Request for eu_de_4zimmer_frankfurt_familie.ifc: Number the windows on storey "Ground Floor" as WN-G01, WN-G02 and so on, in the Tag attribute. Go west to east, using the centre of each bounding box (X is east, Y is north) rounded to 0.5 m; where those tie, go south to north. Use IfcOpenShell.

First a look at what the model holds.

```python
import ifcopenshell
import ifcopenshell.util.element
import ifcopenshell.util.placement

model = ifcopenshell.open("eu_de_4zimmer_frankfurt_familie.ifc")
print(model.schema)
storey = next(s for s in model.by_type("IfcBuildingStorey") if s.Name == "Ground Floor")
windows = [e for e in ifcopenshell.util.element.get_decomposition(storey) if e.is_a("IfcWindow")]
for e in sorted(windows, key=lambda e: e.id()):
    origin = ifcopenshell.util.placement.get_local_placement(e.ObjectPlacement)[:3, 3]
    print(e.id(), e.Tag, e.Name, origin.round(2) + 0.0, sep=" | ")
```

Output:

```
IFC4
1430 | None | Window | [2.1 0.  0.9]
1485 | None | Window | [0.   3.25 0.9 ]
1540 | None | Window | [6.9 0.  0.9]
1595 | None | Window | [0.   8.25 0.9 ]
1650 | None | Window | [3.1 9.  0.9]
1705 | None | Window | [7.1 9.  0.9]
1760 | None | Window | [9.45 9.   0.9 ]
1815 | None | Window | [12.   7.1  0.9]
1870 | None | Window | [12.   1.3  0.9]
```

```python
import ifcopenshell
import ifcopenshell.geom
import ifcopenshell.util.element
import ifcopenshell.util.shape

model = ifcopenshell.open("eu_de_4zimmer_frankfurt_familie.ifc")
settings = ifcopenshell.geom.settings()
settings.set("use-world-coords", True)


def centre(element):
    shape = ifcopenshell.geom.create_shape(settings, element)
    return ifcopenshell.util.shape.get_bbox_centroid(shape.geometry)


storey = next(s for s in model.by_type("IfcBuildingStorey") if s.Name == "Ground Floor")
windows = [e for e in ifcopenshell.util.element.get_decomposition(storey) if e.is_a("IfcWindow")]

# Insertion points can sit at a corner or the storey origin, so sort by the geometry (in metres).
centres = {e: centre(e) for e in windows}
windows.sort(key=lambda e: (round(centres[e][0] / 0.5), centres[e][1]))

for i, e in enumerate(windows, start=1):
    number = f"WN-G{i:02d}"
    e.Tag = number
    print(e.id(), number)

model.write("eu_de_4zimmer_frankfurt_familie-out.ifc")
```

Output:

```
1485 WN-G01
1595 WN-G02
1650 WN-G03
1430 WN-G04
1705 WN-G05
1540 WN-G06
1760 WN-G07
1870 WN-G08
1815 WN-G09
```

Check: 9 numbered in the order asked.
